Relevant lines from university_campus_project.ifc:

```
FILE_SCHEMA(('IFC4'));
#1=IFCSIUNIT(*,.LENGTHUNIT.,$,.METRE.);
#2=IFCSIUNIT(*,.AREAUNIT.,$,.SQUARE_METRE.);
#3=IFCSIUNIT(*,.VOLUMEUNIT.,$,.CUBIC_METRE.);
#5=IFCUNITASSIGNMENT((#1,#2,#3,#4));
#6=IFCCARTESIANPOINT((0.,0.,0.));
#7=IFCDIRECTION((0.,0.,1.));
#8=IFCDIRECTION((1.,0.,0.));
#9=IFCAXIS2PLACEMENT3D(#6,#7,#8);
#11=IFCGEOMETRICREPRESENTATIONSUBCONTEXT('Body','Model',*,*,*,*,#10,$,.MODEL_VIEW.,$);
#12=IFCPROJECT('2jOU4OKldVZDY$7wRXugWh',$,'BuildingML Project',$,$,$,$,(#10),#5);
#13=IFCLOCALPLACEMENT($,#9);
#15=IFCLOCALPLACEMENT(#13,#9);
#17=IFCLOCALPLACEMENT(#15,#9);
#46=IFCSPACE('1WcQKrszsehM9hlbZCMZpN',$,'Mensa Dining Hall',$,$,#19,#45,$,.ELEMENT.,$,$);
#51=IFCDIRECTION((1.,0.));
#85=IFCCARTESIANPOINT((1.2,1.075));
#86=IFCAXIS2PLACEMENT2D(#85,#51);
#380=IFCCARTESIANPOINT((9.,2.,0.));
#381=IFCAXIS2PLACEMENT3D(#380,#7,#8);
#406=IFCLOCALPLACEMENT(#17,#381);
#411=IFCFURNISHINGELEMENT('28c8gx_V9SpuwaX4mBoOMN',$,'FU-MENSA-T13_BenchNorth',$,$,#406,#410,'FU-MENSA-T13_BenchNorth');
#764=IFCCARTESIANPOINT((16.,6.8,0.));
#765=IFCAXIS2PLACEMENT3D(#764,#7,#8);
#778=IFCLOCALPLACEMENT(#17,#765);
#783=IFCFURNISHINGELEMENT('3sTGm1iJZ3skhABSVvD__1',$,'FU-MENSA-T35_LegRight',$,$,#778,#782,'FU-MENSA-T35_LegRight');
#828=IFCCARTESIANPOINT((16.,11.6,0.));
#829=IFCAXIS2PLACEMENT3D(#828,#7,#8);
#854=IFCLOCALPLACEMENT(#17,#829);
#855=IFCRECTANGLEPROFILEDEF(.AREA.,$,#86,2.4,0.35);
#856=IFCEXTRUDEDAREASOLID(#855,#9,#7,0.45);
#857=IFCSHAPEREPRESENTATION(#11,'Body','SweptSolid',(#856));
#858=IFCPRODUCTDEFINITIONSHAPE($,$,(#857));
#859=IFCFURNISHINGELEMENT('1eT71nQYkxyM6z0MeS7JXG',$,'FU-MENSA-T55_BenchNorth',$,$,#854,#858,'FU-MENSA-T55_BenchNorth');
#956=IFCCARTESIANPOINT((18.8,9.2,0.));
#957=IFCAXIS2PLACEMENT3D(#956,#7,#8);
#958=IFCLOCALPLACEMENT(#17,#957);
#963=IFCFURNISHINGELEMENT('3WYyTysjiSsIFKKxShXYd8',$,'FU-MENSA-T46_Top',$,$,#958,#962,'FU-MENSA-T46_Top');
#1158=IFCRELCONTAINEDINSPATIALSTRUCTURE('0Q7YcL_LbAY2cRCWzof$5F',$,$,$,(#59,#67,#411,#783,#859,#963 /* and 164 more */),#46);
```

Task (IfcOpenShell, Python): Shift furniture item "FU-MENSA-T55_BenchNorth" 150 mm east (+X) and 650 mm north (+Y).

```python
import ifcopenshell
import ifcopenshell.api.geometry
import ifcopenshell.util.placement

model = ifcopenshell.open("university_campus_project.ifc")

item = model.by_id(859)
matrix = ifcopenshell.util.placement.get_local_placement(item.ObjectPlacement)
matrix[0, 3] += 0.15
matrix[1, 3] += 0.65
ifcopenshell.api.geometry.edit_object_placement(model, product=item, matrix=matrix, is_si=False)

print(ifcopenshell.util.placement.get_local_placement(item.ObjectPlacement).round(3) + 0.0)

model.write("university_campus_project-out.ifc")
```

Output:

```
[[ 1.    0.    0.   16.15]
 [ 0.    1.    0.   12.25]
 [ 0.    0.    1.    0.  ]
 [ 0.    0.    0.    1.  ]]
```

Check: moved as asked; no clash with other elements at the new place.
